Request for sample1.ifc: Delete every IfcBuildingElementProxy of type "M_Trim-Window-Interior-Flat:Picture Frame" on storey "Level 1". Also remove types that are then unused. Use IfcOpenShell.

First a look at what the model holds.

```python
import ifcopenshell
import ifcopenshell.util.element

model = ifcopenshell.open("sample1.ifc")
print(model.schema)
storey = next(s for s in model.by_type("IfcBuildingStorey") if s.Name == "Level 1")
proxies = [e for e in ifcopenshell.util.element.get_decomposition(storey) if e.is_a("IfcBuildingElementProxy")]
seen = {}
for e in proxies:
    element_type = ifcopenshell.util.element.get_type(e)
    name = element_type.Name if element_type not in (None, e) else None
    seen[name] = seen.get(name, 0) + 1
for name, count in sorted(seen.items(), key=str):
    print(count, "x", name)
```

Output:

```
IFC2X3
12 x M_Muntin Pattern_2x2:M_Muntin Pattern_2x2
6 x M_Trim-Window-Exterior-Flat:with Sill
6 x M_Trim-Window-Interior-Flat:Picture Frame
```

```python
import ifcopenshell
import ifcopenshell.api.root
import ifcopenshell.util.element

model = ifcopenshell.open("sample1.ifc")

storey = next(s for s in model.by_type("IfcBuildingStorey") if s.Name == "Level 1")
proxies = [e for e in ifcopenshell.util.element.get_decomposition(storey) if e.is_a("IfcBuildingElementProxy")]
targets = [e for e in proxies if (t := ifcopenshell.util.element.get_type(e)) not in (None, e) and t.Name == "M_Trim-Window-Interior-Flat:Picture Frame"]
types = {ifcopenshell.util.element.get_type(e) for e in targets} - {None, *targets}

for e in targets:
    ifcopenshell.api.root.remove_product(model, product=e)
print(len(targets), "removed")

unused = [t for t in types if not ifcopenshell.util.element.get_types(t)]
for t in unused:
    ifcopenshell.api.root.remove_product(model, product=t)
print(len(unused), "unused types removed")

model.write("sample1_edited.ifc")
```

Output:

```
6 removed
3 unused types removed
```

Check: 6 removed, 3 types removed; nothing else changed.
